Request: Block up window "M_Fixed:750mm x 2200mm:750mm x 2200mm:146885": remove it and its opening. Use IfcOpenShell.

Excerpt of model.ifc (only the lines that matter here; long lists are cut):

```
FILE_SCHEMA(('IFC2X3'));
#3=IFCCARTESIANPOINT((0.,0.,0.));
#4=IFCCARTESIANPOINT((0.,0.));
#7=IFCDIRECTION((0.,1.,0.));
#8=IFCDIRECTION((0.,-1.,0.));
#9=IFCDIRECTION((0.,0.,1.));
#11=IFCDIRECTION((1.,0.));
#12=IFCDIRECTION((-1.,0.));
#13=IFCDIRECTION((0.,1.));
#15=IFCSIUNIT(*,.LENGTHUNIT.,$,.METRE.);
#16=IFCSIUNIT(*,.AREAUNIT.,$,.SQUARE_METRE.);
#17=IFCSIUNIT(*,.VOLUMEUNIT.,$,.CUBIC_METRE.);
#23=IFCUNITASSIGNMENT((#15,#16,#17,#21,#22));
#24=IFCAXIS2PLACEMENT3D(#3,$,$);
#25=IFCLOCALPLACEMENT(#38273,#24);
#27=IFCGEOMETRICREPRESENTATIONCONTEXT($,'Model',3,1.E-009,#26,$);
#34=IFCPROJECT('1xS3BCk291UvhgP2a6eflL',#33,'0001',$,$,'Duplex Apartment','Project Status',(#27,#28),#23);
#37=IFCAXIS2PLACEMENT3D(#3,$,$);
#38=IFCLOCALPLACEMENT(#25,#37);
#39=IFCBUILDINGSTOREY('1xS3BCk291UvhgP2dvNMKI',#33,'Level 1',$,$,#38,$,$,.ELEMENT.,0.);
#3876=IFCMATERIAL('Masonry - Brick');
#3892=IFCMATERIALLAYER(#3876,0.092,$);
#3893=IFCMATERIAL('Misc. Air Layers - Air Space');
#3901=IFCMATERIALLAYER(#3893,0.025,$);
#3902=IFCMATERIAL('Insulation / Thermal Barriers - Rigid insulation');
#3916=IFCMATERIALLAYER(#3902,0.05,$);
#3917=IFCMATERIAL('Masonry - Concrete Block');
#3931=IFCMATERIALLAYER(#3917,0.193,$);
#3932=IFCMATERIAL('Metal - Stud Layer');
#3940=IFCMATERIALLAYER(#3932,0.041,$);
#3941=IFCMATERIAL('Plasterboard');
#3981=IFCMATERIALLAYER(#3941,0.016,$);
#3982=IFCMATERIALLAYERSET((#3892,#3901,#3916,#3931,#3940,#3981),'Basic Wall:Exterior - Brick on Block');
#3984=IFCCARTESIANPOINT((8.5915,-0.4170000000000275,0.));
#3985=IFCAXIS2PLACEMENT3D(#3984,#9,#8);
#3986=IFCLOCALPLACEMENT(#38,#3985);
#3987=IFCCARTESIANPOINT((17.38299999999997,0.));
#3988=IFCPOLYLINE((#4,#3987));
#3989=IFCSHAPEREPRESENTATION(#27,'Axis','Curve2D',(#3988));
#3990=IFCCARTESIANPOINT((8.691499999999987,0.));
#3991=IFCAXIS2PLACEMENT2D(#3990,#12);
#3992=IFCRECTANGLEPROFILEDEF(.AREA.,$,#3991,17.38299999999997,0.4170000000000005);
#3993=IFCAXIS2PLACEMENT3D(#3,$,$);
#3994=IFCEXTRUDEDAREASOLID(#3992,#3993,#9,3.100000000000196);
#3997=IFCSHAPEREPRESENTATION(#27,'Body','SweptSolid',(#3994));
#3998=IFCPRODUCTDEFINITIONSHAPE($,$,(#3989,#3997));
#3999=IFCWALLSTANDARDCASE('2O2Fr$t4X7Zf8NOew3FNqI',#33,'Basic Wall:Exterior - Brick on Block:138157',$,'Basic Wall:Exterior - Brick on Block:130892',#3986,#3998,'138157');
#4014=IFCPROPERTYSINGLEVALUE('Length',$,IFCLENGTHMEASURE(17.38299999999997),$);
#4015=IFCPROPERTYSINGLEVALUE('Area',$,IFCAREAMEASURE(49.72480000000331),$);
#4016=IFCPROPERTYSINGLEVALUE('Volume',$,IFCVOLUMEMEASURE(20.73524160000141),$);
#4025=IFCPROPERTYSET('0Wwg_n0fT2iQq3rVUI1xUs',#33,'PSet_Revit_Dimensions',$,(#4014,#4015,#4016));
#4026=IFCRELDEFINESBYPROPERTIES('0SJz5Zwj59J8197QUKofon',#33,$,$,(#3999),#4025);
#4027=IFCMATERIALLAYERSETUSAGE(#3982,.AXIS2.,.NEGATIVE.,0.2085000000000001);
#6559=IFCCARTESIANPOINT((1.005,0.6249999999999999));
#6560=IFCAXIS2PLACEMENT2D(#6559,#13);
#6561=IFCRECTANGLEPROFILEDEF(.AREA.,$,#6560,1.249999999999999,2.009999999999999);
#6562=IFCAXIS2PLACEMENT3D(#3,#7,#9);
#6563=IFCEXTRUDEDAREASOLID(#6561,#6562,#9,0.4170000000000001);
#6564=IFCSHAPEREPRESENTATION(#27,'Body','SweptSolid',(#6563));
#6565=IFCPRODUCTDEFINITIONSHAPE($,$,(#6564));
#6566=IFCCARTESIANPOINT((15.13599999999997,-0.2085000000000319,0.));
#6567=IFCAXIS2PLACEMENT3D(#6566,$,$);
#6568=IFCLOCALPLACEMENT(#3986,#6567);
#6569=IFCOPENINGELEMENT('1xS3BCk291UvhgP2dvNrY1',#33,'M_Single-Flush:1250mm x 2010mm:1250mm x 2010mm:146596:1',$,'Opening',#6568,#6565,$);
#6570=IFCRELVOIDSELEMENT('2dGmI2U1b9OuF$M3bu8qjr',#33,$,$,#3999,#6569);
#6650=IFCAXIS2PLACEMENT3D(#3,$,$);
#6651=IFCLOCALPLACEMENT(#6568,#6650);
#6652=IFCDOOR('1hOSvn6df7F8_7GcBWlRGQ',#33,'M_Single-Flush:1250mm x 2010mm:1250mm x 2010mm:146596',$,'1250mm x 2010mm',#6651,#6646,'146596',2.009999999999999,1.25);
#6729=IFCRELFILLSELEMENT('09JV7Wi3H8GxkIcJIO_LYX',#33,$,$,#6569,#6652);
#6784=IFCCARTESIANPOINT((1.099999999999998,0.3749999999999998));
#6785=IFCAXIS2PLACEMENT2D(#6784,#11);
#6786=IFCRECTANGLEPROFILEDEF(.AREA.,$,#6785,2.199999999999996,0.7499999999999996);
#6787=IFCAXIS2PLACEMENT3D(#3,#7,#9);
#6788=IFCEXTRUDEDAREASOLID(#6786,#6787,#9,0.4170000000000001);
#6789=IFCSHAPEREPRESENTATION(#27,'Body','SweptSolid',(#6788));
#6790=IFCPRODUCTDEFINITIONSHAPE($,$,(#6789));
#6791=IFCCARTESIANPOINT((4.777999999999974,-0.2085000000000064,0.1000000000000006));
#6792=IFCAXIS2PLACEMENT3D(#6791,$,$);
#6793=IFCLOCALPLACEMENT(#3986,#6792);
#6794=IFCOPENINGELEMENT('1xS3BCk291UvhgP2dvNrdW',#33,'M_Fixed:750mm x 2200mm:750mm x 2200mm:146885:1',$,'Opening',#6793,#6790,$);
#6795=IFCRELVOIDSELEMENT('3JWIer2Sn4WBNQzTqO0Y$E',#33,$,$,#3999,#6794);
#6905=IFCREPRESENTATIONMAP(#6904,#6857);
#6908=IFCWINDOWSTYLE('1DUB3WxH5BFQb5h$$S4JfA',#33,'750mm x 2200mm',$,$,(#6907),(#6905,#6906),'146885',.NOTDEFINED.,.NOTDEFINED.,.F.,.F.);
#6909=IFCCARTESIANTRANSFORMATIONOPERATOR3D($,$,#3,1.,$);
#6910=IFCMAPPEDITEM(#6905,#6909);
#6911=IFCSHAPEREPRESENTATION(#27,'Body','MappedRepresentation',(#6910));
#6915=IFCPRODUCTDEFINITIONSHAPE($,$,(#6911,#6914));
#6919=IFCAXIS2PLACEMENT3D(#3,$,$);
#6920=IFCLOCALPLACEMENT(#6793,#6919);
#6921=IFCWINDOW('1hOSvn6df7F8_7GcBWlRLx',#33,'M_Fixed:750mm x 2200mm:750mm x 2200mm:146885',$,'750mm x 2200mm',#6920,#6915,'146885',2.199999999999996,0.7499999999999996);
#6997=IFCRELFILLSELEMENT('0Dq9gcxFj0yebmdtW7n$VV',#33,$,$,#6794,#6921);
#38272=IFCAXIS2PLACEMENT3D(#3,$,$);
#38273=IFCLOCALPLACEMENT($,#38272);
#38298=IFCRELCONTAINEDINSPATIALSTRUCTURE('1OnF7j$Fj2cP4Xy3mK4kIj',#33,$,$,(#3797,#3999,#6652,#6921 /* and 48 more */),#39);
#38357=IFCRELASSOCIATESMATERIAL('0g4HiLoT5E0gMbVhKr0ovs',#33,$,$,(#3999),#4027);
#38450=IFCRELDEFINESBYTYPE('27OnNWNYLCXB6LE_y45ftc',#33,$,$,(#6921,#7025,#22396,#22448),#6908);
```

```python
import ifcopenshell
import ifcopenshell.api.feature
import ifcopenshell.api.pset
import ifcopenshell.api.root
import ifcopenshell.geom
import ifcopenshell.util.element
import ifcopenshell.util.shape
import ifcopenshell.util.unit

model = ifcopenshell.open("model.ifc")
area_scale = ifcopenshell.util.unit.calculate_unit_scale(model, "AREAUNIT")
volume_scale = ifcopenshell.util.unit.calculate_unit_scale(model, "VOLUMEUNIT")
settings = ifcopenshell.geom.settings()


def volume(element):
    """Net volume in cubic metres, openings subtracted."""
    shape = ifcopenshell.geom.create_shape(settings, element)
    return ifcopenshell.util.shape.get_volume(shape.geometry)


window = model.by_guid("1hOSvn6df7F8_7GcBWlRLx")
opening = window.FillsVoids[0].RelatingOpeningElement
wall = opening.VoidsElements[0].RelatingBuildingElement
before = volume(wall)

ifcopenshell.api.root.remove_product(model, product=window)
ifcopenshell.api.feature.remove_feature(model, feature=opening)

after = volume(wall)
thickness = 0.417  # wall thickness in metres

# Update the wall's stored quantities.
pset = model.by_id(ifcopenshell.util.element.get_pset(wall, "PSet_Revit_Dimensions", should_inherit=False)["id"])
ifcopenshell.api.pset.edit_pset(model, pset=pset, properties={
    "Area": model.create_entity("IfcAreaMeasure", after / thickness / area_scale),
    "Volume": model.create_entity("IfcVolumeMeasure", after / volume_scale),
})

print(f"wall volume {before:.3f} -> {after:.3f} m3")

model.write("model_v2.ifc")
```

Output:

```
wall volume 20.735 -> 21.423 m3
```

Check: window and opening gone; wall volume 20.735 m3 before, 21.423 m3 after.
